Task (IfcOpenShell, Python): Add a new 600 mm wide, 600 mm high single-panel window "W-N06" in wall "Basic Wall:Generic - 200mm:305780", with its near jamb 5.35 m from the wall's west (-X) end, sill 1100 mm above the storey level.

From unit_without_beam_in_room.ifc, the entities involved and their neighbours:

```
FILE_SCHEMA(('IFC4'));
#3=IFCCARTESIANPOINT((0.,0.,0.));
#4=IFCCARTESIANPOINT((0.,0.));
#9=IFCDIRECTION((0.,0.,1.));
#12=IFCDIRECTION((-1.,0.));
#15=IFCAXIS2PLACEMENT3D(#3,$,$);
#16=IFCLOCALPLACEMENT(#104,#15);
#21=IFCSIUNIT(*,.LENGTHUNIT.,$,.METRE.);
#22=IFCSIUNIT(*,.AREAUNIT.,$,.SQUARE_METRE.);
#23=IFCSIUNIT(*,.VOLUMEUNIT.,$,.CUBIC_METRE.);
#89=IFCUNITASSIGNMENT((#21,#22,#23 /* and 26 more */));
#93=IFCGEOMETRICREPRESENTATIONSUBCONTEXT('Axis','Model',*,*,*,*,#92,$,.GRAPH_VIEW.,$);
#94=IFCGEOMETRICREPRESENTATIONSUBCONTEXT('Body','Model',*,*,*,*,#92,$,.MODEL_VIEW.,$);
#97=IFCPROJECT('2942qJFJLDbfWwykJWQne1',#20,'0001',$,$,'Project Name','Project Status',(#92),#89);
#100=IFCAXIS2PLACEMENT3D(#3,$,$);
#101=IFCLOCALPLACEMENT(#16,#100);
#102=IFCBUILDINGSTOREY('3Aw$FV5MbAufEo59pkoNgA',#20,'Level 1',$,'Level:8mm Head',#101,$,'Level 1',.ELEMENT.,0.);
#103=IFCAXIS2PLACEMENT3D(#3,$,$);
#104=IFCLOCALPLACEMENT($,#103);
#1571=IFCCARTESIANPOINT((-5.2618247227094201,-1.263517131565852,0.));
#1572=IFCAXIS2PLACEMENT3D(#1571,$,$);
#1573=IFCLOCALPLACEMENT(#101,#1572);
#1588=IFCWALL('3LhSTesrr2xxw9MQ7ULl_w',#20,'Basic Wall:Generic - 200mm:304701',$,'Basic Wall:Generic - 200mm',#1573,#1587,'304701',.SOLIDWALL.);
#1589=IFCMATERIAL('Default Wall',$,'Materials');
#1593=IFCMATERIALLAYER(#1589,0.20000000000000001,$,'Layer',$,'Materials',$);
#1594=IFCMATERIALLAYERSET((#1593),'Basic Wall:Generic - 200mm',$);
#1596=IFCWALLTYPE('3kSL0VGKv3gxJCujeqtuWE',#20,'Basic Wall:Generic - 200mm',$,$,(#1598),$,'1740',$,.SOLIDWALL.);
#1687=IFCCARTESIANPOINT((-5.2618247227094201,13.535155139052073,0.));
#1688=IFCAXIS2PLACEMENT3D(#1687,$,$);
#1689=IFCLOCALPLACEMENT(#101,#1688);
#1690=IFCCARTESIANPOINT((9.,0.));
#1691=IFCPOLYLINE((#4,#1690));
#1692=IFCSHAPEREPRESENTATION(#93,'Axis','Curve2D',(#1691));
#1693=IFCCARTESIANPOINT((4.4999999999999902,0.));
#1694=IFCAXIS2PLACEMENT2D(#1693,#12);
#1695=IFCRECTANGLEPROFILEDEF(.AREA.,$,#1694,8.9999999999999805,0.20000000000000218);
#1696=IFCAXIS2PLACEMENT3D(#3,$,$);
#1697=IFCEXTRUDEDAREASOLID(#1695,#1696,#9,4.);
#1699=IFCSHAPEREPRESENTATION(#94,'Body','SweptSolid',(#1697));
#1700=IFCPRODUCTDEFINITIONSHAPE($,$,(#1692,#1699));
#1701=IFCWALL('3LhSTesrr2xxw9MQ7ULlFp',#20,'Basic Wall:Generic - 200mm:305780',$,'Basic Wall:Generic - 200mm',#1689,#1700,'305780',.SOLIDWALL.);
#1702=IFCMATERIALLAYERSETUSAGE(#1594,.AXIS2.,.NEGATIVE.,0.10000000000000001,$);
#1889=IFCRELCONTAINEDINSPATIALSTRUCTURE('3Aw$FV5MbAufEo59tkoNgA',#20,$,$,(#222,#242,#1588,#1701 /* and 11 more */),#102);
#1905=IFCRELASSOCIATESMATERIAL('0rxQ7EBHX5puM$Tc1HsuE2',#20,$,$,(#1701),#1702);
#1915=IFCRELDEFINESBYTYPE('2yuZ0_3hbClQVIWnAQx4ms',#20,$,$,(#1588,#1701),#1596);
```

```python
import numpy as np
import ifcopenshell
import ifcopenshell.api.feature
import ifcopenshell.api.geometry
import ifcopenshell.api.root
import ifcopenshell.api.spatial
import ifcopenshell.geom
import ifcopenshell.util.element
import ifcopenshell.util.placement
import ifcopenshell.util.representation
import ifcopenshell.util.shape
import ifcopenshell.util.unit

model = ifcopenshell.open("unit_without_beam_in_room.ifc")
unit_scale = ifcopenshell.util.unit.calculate_unit_scale(model)
settings = ifcopenshell.geom.settings()


def volume(element):
    """Net volume in cubic metres, openings subtracted."""
    shape = ifcopenshell.geom.create_shape(settings, element)
    return ifcopenshell.util.shape.get_volume(shape.geometry)


wall = model.by_guid("3LhSTesrr2xxw9MQ7ULlFp")
storey = ifcopenshell.util.element.get_container(wall, ifc_class="IfcBuildingStorey")
context = ifcopenshell.util.representation.get_context(model, "Model", "Body", "MODEL_VIEW")
before = volume(wall)

width, height, from_end, sill = 0.6, 0.6, 5.35, 1.1  # metres

# The wall runs along its own X axis, and the end named is its -X end.
wall_shape = ifcopenshell.geom.create_shape(settings, wall)
x, y, z = ifcopenshell.util.shape.get_vertices(wall_shape.geometry).T
start = x.min() + from_end
face, thickness = float(y.min()), float(y.max() - y.min())
wall_matrix = ifcopenshell.util.placement.get_local_placement(wall.ObjectPlacement)
level = ifcopenshell.util.placement.get_local_placement(storey.ObjectPlacement)[2, 3]


def in_wall(x, y):
    """Placement at x, y metres in the wall's axes, at sill height."""
    matrix = wall_matrix.copy()
    matrix[:, 3] = wall_matrix @ np.array([x / unit_scale, y / unit_scale, 0.0, 1.0])
    matrix[2, 3] = level + sill / unit_scale
    return matrix


# Opening: a box that overshoots both wall faces by 50 mm.
opening = ifcopenshell.api.root.create_entity(model, ifc_class="IfcOpeningElement", predefined_type="OPENING")
box = ifcopenshell.api.geometry.add_wall_representation(
    model, context=context, length=width, height=height, thickness=thickness + 0.1
)
ifcopenshell.api.geometry.assign_representation(model, product=opening, representation=box)
ifcopenshell.api.geometry.edit_object_placement(model, product=opening, matrix=in_wall(start, face - 0.05), is_si=False)
ifcopenshell.api.feature.add_feature(model, feature=opening, element=wall)

window = ifcopenshell.api.root.create_entity(model, ifc_class="IfcWindow", name="W-N06", predefined_type="WINDOW")
window.OverallWidth, window.OverallHeight = width / unit_scale, height / unit_scale
window.PartitioningType = "SINGLE_PANEL"
body = ifcopenshell.api.geometry.add_window_representation(
    model,
    context=context,
    overall_width=window.OverallWidth,
    overall_height=window.OverallHeight,
    partition_type="SINGLE_PANEL",
)
ifcopenshell.api.geometry.assign_representation(model, product=window, representation=body)
ifcopenshell.api.spatial.assign_container(model, products=[window], relating_structure=storey)
ifcopenshell.api.feature.add_filling(model, opening=opening, element=window)

# Centre the window in the wall's thickness.
ifcopenshell.api.geometry.edit_object_placement(model, product=window, matrix=in_wall(start, face), is_si=False)
window_shape = ifcopenshell.geom.create_shape(settings, window)
depth = ifcopenshell.util.shape.get_vertices(window_shape.geometry)[:, 1]
offset = face + thickness / 2 - (depth.min() + depth.max()) / 2
ifcopenshell.api.geometry.edit_object_placement(model, product=window, matrix=in_wall(start, offset), is_si=False)

after = volume(wall)

print(f"wall volume {before:.3f} -> {after:.3f} m3")

model.write("unit_without_beam_in_room_edited.ifc")
```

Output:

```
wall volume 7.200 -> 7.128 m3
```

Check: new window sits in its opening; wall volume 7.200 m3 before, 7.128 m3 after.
